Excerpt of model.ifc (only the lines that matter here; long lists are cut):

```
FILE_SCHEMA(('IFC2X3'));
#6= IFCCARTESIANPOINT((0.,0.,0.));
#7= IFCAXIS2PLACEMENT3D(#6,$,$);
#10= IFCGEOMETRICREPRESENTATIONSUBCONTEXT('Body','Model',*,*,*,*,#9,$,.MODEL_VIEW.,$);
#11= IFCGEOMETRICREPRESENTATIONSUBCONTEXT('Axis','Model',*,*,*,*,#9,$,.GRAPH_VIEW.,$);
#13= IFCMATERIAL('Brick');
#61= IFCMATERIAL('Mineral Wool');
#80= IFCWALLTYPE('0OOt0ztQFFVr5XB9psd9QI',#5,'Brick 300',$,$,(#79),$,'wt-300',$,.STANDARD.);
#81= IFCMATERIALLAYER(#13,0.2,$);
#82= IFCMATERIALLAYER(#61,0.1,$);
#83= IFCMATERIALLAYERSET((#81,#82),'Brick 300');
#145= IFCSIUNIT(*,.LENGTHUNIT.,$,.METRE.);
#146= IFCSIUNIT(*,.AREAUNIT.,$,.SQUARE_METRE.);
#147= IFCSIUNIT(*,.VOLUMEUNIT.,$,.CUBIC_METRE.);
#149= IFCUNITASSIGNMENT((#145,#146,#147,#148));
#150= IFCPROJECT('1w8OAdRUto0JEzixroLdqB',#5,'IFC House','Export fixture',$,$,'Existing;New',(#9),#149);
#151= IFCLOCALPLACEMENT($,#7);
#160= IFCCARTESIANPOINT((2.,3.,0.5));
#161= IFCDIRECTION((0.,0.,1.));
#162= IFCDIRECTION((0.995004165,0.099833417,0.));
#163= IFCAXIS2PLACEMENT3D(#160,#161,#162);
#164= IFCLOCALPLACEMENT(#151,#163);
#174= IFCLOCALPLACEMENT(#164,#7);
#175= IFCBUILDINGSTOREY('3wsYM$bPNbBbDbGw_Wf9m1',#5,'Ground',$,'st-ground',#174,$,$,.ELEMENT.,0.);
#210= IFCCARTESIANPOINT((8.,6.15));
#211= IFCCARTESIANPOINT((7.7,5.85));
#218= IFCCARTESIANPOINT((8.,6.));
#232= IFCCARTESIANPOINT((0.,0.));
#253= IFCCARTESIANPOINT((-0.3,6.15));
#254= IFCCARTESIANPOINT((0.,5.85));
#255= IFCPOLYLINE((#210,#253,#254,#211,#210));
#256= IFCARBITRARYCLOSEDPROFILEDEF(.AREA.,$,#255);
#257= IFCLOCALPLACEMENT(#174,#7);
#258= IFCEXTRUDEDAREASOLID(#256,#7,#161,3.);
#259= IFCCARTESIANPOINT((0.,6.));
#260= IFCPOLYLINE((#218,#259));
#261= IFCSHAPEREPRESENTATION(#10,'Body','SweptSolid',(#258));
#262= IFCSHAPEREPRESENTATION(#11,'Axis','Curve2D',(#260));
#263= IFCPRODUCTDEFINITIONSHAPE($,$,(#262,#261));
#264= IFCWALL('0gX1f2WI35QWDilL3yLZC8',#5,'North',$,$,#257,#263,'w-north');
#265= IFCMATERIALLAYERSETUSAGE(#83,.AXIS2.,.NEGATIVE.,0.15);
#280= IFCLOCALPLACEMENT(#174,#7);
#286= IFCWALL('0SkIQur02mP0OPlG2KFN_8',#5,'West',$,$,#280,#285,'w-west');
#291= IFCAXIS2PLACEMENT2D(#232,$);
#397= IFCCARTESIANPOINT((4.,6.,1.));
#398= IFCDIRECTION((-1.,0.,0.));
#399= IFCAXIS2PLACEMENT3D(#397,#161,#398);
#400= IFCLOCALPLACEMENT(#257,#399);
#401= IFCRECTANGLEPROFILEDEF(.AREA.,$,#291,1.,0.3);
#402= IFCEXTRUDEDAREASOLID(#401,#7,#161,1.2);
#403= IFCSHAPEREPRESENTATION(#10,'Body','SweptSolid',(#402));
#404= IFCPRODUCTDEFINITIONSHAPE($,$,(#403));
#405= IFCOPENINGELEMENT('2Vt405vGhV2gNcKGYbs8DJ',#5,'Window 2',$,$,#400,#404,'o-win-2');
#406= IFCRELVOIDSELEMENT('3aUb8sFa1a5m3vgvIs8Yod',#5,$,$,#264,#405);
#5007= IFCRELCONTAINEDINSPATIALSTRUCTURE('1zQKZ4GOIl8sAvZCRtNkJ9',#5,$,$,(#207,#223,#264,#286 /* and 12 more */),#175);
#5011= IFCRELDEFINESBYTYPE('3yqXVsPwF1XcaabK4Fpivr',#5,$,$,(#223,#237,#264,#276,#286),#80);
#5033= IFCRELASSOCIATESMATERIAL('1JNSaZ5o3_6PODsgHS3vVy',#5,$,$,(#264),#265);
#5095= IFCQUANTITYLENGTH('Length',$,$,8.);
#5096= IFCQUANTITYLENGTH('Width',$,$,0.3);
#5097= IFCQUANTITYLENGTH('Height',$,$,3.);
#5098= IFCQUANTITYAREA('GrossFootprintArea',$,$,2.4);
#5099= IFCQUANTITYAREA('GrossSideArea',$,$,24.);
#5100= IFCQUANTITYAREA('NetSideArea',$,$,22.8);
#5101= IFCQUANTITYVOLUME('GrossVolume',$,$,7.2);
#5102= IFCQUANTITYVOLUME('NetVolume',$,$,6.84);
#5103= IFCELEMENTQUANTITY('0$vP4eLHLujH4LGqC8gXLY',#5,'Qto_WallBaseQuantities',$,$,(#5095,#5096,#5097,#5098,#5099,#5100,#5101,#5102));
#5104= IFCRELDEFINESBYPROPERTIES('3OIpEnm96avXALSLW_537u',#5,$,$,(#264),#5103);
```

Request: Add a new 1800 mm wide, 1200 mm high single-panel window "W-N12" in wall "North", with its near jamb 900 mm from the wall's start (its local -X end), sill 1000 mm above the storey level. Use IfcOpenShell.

```python
import numpy as np
import ifcopenshell
import ifcopenshell.api.feature
import ifcopenshell.api.geometry
import ifcopenshell.api.pset
import ifcopenshell.api.root
import ifcopenshell.api.spatial
import ifcopenshell.api.type
import ifcopenshell.geom
import ifcopenshell.util.element
import ifcopenshell.util.placement
import ifcopenshell.util.representation
import ifcopenshell.util.shape
import ifcopenshell.util.unit

model = ifcopenshell.open("model.ifc")
unit_scale = ifcopenshell.util.unit.calculate_unit_scale(model)
area_scale = ifcopenshell.util.unit.calculate_unit_scale(model, "AREAUNIT")
volume_scale = ifcopenshell.util.unit.calculate_unit_scale(model, "VOLUMEUNIT")
settings = ifcopenshell.geom.settings()


def volume(element):
    """Net volume in cubic metres, openings subtracted."""
    shape = ifcopenshell.geom.create_shape(settings, element)
    return ifcopenshell.util.shape.get_volume(shape.geometry)


wall = model.by_guid("0gX1f2WI35QWDilL3yLZC8")
storey = ifcopenshell.util.element.get_container(wall, ifc_class="IfcBuildingStorey")
context = ifcopenshell.util.representation.get_context(model, "Model", "Body", "MODEL_VIEW")
before = volume(wall)

width, height, from_end, sill = 1.8, 1.2, 0.9, 1  # metres

# The wall runs along its own X axis, and the end named is its -X end.
wall_shape = ifcopenshell.geom.create_shape(settings, wall)
x, y, z = ifcopenshell.util.shape.get_vertices(wall_shape.geometry).T
start = x.min() + from_end
face, thickness = float(y.min()), float(y.max() - y.min())
wall_matrix = ifcopenshell.util.placement.get_local_placement(wall.ObjectPlacement)
level = ifcopenshell.util.placement.get_local_placement(storey.ObjectPlacement)[2, 3]


def in_wall(x, y):
    """Placement at x, y metres in the wall's axes, at sill height."""
    matrix = wall_matrix.copy()
    matrix[:, 3] = wall_matrix @ np.array([x / unit_scale, y / unit_scale, 0.0, 1.0])
    matrix[2, 3] = level + sill / unit_scale
    return matrix


# Opening: a box that overshoots both wall faces by 50 mm.
opening = ifcopenshell.api.root.create_entity(model, ifc_class="IfcOpeningElement")
box = ifcopenshell.api.geometry.add_wall_representation(
    model, context=context, length=width, height=height, thickness=thickness + 0.1
)
ifcopenshell.api.geometry.assign_representation(model, product=opening, representation=box)
ifcopenshell.api.geometry.edit_object_placement(model, product=opening, matrix=in_wall(start, face - 0.05), is_si=False)
ifcopenshell.api.feature.add_feature(model, feature=opening, element=wall)

window = ifcopenshell.api.root.create_entity(model, ifc_class="IfcWindow", name="W-N12")
window.OverallWidth, window.OverallHeight = width / unit_scale, height / unit_scale
body = ifcopenshell.api.geometry.add_window_representation(
    model,
    context=context,
    overall_width=window.OverallWidth,
    overall_height=window.OverallHeight,
    partition_type="SINGLE_PANEL",
)
ifcopenshell.api.geometry.assign_representation(model, product=window, representation=body)
ifcopenshell.api.spatial.assign_container(model, products=[window], relating_structure=storey)
fills = ifcopenshell.api.feature.add_filling(model, opening=opening, element=window)
fills.OwnerHistory = window.OwnerHistory  # required in IFC2X3

# IFC2X3 keeps the operation on the window style.
style = ifcopenshell.api.root.create_entity(model, ifc_class="IfcWindowStyle", name="W-N12")
style.OperationType, style.ConstructionType = "SINGLE_PANEL", "NOTDEFINED"
style.ParameterTakesPrecedence = style.Sizeable = False
ifcopenshell.api.type.assign_type(model, related_objects=[window], relating_type=style)

# Centre the window in the wall's thickness.
ifcopenshell.api.geometry.edit_object_placement(model, product=window, matrix=in_wall(start, face), is_si=False)
window_shape = ifcopenshell.geom.create_shape(settings, window)
depth = ifcopenshell.util.shape.get_vertices(window_shape.geometry)[:, 1]
offset = face + thickness / 2 - (depth.min() + depth.max()) / 2
ifcopenshell.api.geometry.edit_object_placement(model, product=window, matrix=in_wall(start, offset), is_si=False)

after = volume(wall)

# Update the wall's stored quantities.
qto = model.by_id(ifcopenshell.util.element.get_pset(wall, "Qto_WallBaseQuantities", should_inherit=False)["id"])
ifcopenshell.api.pset.edit_qto(model, qto=qto, properties={
    "NetSideArea": after / thickness / area_scale,
    "NetVolume": after / volume_scale,
})

print(f"wall volume {before:.3f} -> {after:.3f} m3")

model.write("model_v2.ifc")
```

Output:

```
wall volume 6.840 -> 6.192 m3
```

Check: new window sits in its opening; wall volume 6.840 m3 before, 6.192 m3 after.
